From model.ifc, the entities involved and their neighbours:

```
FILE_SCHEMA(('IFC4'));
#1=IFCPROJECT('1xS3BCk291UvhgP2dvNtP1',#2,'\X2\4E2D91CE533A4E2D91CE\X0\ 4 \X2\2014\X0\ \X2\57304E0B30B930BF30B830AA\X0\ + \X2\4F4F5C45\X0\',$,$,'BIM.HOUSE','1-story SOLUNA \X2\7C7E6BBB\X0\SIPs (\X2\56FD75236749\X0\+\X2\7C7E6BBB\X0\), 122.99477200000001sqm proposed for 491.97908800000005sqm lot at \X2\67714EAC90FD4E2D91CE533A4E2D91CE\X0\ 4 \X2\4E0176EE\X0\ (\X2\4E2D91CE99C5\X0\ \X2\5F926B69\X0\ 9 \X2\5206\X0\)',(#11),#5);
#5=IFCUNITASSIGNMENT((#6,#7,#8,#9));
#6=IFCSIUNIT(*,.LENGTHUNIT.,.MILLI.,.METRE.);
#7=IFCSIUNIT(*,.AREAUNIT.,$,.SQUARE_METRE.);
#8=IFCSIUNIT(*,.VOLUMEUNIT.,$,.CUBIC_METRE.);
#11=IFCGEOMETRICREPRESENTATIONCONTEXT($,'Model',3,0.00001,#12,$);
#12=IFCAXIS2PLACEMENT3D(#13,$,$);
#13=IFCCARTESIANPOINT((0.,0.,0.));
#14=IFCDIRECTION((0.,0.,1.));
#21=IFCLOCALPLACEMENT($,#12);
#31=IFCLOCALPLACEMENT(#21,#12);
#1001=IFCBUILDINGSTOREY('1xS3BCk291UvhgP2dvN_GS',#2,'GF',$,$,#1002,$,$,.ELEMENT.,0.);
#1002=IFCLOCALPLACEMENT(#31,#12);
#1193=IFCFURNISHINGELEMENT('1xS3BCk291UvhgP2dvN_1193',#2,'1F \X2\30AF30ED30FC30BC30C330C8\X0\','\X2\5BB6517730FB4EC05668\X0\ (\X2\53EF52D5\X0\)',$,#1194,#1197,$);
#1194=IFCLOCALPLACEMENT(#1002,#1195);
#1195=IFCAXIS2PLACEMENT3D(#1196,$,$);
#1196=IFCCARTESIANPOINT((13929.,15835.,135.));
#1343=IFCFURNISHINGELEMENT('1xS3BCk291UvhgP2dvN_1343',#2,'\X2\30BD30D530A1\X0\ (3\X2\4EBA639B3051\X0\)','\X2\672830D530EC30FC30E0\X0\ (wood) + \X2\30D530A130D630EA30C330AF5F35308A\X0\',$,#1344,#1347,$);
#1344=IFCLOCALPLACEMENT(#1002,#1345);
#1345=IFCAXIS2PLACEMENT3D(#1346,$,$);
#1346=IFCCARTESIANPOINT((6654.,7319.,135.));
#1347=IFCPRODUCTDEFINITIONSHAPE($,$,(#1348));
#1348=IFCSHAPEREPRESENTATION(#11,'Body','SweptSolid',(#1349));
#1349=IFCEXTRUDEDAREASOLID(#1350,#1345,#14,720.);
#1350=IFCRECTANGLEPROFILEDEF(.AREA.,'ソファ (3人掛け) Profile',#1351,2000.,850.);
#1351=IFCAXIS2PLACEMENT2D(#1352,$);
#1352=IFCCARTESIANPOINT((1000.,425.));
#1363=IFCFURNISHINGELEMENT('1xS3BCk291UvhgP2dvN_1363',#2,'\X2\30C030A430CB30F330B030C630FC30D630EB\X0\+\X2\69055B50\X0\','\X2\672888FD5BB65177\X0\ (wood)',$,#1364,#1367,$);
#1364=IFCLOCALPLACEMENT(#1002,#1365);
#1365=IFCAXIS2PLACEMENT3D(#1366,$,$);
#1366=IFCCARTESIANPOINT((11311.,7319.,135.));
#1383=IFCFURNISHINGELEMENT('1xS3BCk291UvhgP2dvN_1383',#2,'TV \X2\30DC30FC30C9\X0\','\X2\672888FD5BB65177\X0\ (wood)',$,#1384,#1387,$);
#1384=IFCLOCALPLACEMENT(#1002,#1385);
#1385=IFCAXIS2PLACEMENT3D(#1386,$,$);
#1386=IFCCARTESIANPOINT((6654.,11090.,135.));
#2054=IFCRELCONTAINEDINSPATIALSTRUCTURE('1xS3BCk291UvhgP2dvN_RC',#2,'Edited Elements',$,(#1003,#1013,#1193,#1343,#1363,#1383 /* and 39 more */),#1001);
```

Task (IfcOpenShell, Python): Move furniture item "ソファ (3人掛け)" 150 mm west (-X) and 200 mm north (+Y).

```python
import ifcopenshell
import ifcopenshell.api.geometry
import ifcopenshell.util.placement
import ifcopenshell.util.unit

model = ifcopenshell.open("model.ifc")
unit_scale = ifcopenshell.util.unit.calculate_unit_scale(model)

item = model.by_guid("1xS3BCk291UvhgP2dvN_1343")
matrix = ifcopenshell.util.placement.get_local_placement(item.ObjectPlacement)
matrix[0, 3] -= 0.15 / unit_scale
matrix[1, 3] += 0.2 / unit_scale
ifcopenshell.api.geometry.edit_object_placement(model, product=item, matrix=matrix, is_si=False)

print(ifcopenshell.util.placement.get_local_placement(item.ObjectPlacement).round(3) + 0.0)

model.write("model_rev.ifc")
```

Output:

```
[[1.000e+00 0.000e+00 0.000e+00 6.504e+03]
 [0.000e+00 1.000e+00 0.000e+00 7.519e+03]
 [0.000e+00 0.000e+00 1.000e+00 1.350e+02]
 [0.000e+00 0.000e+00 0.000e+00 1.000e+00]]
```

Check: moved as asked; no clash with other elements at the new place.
